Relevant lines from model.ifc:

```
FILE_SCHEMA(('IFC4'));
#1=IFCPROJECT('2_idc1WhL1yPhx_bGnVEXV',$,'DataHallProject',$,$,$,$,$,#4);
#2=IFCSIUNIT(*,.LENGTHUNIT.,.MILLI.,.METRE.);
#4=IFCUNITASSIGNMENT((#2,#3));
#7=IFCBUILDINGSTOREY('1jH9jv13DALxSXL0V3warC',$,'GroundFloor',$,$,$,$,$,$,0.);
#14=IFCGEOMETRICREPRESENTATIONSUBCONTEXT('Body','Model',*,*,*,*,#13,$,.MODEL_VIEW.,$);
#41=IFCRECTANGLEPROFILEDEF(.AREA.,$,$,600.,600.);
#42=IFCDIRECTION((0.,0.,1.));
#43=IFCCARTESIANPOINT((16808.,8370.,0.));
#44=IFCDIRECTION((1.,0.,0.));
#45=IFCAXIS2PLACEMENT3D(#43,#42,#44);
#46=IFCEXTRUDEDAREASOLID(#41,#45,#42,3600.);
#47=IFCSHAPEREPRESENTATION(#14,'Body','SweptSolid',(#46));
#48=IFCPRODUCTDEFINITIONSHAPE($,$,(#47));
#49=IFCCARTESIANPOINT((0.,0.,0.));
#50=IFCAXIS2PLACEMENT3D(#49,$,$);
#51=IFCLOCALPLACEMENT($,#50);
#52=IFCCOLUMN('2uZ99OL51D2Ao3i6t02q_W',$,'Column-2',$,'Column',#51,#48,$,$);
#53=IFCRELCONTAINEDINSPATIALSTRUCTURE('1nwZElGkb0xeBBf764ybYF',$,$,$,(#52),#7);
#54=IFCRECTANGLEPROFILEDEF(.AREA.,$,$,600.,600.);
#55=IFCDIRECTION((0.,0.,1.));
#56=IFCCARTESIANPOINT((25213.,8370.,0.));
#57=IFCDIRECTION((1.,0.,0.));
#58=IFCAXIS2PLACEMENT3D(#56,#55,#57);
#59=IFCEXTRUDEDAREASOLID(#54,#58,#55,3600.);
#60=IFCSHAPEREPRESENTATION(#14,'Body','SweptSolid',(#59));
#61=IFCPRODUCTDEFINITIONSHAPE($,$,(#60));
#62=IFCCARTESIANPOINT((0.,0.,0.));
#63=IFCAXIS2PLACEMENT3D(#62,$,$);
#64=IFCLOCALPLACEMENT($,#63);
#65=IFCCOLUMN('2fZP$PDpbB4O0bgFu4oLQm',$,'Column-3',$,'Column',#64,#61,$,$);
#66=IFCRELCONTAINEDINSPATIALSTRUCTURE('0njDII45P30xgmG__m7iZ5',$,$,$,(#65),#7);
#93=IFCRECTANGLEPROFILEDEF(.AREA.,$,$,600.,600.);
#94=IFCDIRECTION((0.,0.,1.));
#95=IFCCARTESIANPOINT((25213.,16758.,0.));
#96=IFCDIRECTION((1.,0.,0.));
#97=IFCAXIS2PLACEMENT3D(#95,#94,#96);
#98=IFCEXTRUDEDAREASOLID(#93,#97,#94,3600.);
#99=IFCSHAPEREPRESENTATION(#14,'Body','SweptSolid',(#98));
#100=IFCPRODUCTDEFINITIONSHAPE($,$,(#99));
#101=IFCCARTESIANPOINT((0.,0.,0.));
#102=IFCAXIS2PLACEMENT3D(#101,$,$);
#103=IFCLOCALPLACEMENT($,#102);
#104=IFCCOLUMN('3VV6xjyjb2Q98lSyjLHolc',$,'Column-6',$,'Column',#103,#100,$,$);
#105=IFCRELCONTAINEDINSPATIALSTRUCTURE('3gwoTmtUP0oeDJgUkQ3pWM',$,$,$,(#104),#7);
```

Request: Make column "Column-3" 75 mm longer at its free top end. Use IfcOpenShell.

```python
import ifcopenshell
import ifcopenshell.util.representation
import ifcopenshell.util.unit

model = ifcopenshell.open("model.ifc")
unit_scale = ifcopenshell.util.unit.calculate_unit_scale(model)

member = model.by_id(65)
change = 0.075 / unit_scale

# The extrusion runs towards the end named, so only its depth changes.
body = ifcopenshell.util.representation.get_representation(member, "Model", "Body")
solid = body.Items[0]
old_length = solid.Depth
solid.Depth += change

print(f"length {old_length:g} -> {solid.Depth:g}")

model.write("model-out.ifc")
```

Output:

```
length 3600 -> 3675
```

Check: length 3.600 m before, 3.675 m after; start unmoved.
